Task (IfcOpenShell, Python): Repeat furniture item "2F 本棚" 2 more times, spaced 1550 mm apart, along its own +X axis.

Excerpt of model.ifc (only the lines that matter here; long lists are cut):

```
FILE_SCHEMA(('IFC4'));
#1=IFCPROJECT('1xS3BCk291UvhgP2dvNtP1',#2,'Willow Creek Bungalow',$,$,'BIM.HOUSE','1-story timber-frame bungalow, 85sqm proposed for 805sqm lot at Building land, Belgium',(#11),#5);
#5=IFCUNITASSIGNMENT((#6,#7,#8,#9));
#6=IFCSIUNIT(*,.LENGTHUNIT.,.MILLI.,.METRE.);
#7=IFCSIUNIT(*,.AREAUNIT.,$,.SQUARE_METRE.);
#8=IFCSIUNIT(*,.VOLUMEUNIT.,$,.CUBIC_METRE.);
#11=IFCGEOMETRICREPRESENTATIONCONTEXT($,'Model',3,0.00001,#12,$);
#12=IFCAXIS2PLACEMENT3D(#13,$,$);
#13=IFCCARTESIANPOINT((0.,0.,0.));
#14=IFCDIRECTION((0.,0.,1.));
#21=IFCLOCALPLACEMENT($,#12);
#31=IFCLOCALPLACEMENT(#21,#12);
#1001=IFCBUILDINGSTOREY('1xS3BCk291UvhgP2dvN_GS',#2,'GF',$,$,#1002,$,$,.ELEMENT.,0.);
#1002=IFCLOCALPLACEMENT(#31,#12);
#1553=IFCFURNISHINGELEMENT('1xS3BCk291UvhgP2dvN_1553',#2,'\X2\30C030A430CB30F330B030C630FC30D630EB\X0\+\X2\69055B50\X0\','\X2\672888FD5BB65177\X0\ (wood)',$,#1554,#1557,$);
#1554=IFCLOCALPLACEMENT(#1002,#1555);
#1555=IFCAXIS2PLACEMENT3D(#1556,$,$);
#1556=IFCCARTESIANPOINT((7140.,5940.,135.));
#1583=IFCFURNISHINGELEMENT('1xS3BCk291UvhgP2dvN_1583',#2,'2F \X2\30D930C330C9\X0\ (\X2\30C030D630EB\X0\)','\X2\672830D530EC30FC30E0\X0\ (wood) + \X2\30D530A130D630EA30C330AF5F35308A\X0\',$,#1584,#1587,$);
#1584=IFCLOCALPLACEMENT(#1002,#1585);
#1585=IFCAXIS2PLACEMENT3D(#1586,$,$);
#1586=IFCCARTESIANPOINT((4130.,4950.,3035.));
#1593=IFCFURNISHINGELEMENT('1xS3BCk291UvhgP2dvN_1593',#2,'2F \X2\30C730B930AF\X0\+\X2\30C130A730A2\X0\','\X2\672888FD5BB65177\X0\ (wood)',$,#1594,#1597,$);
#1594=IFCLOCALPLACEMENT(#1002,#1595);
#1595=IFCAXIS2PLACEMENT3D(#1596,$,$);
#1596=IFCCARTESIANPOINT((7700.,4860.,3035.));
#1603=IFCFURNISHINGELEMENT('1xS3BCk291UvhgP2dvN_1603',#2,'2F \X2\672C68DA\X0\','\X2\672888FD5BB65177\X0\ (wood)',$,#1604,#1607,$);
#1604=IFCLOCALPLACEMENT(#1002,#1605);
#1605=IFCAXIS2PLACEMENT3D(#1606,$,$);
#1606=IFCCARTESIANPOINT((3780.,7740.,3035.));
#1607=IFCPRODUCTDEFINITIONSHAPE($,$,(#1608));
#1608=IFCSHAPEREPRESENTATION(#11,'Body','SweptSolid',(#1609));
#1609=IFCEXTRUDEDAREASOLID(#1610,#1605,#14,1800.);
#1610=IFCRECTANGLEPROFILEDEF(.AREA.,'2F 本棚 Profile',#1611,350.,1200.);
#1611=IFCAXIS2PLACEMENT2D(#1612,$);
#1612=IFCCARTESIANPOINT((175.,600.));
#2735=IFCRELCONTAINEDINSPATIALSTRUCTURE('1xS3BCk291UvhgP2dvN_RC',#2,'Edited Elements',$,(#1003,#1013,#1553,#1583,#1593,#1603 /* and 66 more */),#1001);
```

```python
import ifcopenshell
import ifcopenshell.api.geometry
import ifcopenshell.api.root
import ifcopenshell.util.element
import ifcopenshell.util.placement
import ifcopenshell.util.unit

model = ifcopenshell.open("model.ifc")
unit_scale = ifcopenshell.util.unit.calculate_unit_scale(model)


def reuse_history(source, copy):
    """copy_class also copies each property set's owner history, people and application; keep the originals."""
    for rel in copy.IsDefinedBy:
        if rel.is_a("IfcRelDefinesByProperties") and (history := rel.RelatingPropertyDefinition.OwnerHistory):
            rel.RelatingPropertyDefinition.OwnerHistory = source.OwnerHistory
            ifcopenshell.util.element.remove_deep2(model, history)


source = model.by_guid("1xS3BCk291UvhgP2dvN_1603")
base = ifcopenshell.util.placement.get_local_placement(source.ObjectPlacement)
step = base[:3, 0] * 1.55 / unit_scale

for i in range(1, 3):
    copy = ifcopenshell.api.root.copy_class(model, product=source)
    copy.Representation = ifcopenshell.util.element.copy_deep(
        model, source.Representation, exclude=["IfcGeometricRepresentationContext", "IfcRepresentationMap"]
    )
    reuse_history(source, copy)
    matrix = base.copy()
    matrix[:3, 3] += i * step
    print("added at", matrix[:3, 3].round(3) + 0.0)
    ifcopenshell.api.geometry.edit_object_placement(model, product=copy, matrix=matrix, is_si=False)

model.write("model_updated.ifc")
```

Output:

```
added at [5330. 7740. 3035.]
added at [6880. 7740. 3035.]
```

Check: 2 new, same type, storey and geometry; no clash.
